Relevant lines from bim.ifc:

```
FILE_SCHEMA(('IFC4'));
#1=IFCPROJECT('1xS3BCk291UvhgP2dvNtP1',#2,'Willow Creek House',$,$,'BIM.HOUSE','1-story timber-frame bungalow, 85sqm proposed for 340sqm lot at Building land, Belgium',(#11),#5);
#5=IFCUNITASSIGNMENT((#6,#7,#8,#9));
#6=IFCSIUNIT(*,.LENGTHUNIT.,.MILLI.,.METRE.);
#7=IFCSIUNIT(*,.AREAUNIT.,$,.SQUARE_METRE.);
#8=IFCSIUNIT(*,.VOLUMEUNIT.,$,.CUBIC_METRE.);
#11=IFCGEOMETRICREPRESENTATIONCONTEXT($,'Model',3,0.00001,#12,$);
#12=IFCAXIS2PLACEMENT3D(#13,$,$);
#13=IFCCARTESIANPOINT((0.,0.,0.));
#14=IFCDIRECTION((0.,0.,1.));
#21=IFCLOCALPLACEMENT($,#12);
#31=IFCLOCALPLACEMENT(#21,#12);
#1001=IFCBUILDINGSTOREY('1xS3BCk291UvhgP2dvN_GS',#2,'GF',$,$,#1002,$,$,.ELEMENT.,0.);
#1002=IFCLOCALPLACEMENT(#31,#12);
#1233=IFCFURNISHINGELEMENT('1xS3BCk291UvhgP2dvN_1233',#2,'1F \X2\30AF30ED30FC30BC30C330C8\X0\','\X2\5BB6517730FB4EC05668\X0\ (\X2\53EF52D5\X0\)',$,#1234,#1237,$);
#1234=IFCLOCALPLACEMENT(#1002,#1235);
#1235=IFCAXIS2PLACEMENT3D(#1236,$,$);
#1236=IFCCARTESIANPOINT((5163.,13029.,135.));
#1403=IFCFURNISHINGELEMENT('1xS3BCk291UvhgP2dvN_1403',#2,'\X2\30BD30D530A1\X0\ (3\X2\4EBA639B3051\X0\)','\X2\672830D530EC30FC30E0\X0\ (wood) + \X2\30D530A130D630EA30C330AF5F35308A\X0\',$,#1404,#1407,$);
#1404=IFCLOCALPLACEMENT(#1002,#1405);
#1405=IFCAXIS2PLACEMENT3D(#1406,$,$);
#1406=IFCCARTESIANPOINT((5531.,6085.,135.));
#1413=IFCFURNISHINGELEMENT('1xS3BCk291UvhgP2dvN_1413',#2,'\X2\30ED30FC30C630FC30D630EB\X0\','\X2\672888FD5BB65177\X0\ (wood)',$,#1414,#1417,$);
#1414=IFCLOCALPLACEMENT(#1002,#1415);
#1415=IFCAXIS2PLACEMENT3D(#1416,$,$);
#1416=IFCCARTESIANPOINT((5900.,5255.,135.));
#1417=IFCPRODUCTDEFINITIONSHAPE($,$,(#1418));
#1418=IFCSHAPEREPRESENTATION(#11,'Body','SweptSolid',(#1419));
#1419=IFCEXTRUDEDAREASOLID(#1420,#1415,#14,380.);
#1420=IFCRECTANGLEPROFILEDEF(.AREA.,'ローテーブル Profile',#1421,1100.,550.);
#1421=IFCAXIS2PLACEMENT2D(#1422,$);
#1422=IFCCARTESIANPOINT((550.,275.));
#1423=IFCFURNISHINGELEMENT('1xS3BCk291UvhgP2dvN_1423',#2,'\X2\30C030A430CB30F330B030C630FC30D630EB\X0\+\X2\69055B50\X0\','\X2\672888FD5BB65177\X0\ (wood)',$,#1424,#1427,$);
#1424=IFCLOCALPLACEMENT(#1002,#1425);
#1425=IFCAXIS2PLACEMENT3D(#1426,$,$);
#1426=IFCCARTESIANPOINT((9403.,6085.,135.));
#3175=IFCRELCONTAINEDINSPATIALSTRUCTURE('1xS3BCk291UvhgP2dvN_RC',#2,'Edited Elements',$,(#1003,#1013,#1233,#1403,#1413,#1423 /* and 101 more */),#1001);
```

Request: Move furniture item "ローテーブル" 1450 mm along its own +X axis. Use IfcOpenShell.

```python
import ifcopenshell
import ifcopenshell.api.geometry
import ifcopenshell.util.placement

model = ifcopenshell.open("bim.ifc")

item = model.by_id(1413)
matrix = ifcopenshell.util.placement.get_local_placement(item.ObjectPlacement)
matrix[:3, 3] += matrix[:3, 0] * 1450.0
ifcopenshell.api.geometry.edit_object_placement(model, product=item, matrix=matrix, is_si=False)

print(ifcopenshell.util.placement.get_local_placement(item.ObjectPlacement).round(3) + 0.0)

model.write("bim_rev.ifc")
```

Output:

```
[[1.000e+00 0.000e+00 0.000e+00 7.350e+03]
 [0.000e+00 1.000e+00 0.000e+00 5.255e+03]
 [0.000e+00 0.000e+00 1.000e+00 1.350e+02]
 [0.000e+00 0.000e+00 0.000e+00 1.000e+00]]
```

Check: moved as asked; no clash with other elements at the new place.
